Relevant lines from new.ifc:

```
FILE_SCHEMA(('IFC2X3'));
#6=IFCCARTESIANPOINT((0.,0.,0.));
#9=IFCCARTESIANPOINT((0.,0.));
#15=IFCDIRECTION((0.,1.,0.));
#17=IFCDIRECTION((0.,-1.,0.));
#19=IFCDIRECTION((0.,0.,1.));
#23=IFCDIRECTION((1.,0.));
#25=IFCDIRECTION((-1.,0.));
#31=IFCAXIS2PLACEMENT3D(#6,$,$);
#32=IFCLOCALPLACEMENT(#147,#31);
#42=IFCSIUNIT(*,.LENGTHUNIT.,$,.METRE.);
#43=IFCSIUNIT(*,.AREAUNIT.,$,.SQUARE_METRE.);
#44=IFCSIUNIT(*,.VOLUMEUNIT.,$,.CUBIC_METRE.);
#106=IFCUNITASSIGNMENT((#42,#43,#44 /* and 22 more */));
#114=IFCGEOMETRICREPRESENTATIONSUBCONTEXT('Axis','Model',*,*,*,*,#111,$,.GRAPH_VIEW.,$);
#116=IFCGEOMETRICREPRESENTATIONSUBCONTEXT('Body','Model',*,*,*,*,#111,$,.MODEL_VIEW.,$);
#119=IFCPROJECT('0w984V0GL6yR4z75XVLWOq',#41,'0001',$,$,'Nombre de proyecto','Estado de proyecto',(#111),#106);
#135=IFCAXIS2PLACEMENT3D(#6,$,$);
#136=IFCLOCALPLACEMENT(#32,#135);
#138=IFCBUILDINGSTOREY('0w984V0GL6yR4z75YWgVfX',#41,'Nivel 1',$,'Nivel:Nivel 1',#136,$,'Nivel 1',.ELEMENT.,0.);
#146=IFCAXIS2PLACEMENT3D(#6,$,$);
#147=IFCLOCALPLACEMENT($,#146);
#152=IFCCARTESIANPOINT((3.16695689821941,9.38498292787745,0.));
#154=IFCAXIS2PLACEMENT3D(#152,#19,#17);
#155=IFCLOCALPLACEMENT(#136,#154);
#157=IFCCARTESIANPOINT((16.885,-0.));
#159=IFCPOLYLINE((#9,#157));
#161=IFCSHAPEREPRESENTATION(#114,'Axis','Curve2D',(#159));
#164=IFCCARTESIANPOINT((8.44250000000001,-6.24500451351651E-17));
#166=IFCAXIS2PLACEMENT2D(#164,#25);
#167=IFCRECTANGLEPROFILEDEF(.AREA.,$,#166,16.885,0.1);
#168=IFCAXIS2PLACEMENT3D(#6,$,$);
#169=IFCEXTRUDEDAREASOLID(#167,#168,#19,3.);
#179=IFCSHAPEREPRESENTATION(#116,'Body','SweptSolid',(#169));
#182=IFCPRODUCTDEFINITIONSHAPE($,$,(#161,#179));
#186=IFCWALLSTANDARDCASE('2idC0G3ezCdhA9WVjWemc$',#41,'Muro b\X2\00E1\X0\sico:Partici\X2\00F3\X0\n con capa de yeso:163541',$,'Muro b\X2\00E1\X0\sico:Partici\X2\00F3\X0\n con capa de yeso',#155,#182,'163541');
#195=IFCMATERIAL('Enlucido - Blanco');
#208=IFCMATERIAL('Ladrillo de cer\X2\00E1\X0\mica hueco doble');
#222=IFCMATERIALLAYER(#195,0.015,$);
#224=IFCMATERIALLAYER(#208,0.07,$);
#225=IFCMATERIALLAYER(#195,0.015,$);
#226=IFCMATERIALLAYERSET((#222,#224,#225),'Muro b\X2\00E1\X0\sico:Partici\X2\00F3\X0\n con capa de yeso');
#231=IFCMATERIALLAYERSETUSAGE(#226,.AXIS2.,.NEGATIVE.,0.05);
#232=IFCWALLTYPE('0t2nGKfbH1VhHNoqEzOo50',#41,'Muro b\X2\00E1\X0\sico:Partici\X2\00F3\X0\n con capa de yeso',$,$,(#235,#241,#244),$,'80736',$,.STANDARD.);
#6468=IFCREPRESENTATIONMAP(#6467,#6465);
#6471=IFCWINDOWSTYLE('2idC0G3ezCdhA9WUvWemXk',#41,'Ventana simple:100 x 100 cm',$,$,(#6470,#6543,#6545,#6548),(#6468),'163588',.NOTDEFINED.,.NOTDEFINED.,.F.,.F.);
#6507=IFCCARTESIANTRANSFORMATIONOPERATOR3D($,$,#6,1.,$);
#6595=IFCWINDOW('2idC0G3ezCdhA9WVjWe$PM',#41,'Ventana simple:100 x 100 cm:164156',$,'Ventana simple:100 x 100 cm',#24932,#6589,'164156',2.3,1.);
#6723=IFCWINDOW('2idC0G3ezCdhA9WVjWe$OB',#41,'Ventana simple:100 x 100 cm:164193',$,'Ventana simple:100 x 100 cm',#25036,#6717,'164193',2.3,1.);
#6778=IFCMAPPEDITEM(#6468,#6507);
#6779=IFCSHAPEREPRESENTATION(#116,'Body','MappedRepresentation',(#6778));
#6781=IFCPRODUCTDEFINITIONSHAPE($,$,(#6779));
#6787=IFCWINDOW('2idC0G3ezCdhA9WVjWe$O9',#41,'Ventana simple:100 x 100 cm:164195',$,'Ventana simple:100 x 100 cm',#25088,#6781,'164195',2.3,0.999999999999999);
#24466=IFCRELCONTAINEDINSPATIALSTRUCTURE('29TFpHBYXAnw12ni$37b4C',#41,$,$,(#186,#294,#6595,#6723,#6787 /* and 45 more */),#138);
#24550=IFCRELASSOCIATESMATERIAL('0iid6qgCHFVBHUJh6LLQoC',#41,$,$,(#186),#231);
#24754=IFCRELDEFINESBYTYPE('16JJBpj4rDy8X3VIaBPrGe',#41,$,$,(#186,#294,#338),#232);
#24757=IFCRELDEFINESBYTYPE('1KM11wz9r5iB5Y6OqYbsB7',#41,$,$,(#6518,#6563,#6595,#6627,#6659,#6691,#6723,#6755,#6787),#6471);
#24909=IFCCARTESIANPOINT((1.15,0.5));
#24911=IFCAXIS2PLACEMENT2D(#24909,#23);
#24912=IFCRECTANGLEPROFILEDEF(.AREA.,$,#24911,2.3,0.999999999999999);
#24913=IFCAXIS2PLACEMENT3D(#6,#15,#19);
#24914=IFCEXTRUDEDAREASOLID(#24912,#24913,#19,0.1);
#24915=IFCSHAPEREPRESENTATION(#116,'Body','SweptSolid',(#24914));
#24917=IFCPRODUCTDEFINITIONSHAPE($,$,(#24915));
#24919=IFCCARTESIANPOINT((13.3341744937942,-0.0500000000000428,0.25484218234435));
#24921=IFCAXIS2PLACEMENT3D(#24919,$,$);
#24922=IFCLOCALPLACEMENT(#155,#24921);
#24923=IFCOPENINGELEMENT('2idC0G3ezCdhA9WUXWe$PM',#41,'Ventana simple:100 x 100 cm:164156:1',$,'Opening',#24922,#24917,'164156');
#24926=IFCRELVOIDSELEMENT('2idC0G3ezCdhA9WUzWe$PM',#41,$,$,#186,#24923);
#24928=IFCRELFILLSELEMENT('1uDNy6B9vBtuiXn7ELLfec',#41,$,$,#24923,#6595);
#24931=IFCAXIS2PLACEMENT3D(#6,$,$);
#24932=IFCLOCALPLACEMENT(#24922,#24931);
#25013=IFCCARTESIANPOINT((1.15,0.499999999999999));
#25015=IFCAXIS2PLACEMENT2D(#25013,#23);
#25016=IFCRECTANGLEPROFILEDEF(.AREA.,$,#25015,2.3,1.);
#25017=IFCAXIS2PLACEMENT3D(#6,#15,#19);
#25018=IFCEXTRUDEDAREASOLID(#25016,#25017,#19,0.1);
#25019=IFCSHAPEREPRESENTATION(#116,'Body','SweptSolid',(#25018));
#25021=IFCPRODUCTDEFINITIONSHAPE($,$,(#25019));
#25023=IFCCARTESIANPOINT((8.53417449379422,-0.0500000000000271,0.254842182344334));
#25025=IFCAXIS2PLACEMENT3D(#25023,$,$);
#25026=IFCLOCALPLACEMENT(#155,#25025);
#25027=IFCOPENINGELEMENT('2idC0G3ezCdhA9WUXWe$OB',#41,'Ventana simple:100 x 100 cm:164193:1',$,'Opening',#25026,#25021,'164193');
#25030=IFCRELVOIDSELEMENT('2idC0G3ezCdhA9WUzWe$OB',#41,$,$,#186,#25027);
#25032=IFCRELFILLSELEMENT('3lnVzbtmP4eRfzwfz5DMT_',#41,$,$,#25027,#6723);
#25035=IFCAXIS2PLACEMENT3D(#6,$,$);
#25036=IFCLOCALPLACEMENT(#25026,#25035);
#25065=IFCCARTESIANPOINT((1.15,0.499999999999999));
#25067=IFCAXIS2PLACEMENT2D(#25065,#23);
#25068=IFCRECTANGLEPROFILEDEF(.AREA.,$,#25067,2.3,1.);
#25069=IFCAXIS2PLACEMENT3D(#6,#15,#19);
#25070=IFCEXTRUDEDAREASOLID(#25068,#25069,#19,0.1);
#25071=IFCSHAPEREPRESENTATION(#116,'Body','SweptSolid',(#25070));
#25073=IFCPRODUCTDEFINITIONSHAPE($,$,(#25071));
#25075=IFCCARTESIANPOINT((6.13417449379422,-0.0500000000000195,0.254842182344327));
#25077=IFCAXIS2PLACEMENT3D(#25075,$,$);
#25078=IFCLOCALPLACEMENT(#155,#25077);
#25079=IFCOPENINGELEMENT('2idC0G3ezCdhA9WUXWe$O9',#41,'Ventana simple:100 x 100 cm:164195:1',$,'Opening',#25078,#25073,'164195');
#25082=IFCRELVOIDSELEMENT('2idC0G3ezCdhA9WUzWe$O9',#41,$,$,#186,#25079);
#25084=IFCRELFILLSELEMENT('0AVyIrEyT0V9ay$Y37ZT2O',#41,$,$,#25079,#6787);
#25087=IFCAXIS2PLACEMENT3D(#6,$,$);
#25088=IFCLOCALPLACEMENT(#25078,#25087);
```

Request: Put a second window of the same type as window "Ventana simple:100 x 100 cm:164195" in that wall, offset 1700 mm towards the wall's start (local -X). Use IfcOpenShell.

```python
import ifcopenshell
import ifcopenshell.api.feature
import ifcopenshell.api.geometry
import ifcopenshell.api.root
import ifcopenshell.geom
import ifcopenshell.util.element
import ifcopenshell.util.placement
import ifcopenshell.util.shape

model = ifcopenshell.open("new.ifc")
settings = ifcopenshell.geom.settings()


def volume(element):
    """Net volume in cubic metres, openings subtracted."""
    shape = ifcopenshell.geom.create_shape(settings, element)
    return ifcopenshell.util.shape.get_volume(shape.geometry)


def reuse_history(source, copy):
    """copy_class also copies each property set's owner history, people and application; keep the originals."""
    for rel in copy.IsDefinedBy:
        if rel.is_a("IfcRelDefinesByProperties") and (history := rel.RelatingPropertyDefinition.OwnerHistory):
            rel.RelatingPropertyDefinition.OwnerHistory = source.OwnerHistory
            ifcopenshell.util.element.remove_deep2(model, history)


window = model.by_id(6787)
opening = window.FillsVoids[0].RelatingOpeningElement
wall = opening.VoidsElements[0].RelatingBuildingElement
before = volume(wall)
shift = ifcopenshell.util.placement.get_local_placement(wall.ObjectPlacement)[:3, 0] * -1.7

# copy_class copies the void relationship, type, container and properties, but no geometry.
new_opening = ifcopenshell.api.root.copy_class(model, product=opening)
new_opening.Representation = ifcopenshell.util.element.copy_deep(
    model, opening.Representation, exclude=["IfcGeometricRepresentationContext", "IfcRepresentationMap"]
)
new_opening.Name = "Ventana simple:100 x 100 cm"
new_opening.Tag = None
new_window = ifcopenshell.api.root.copy_class(model, product=window)
new_window.Representation = ifcopenshell.util.element.copy_deep(
    model, window.Representation, exclude=["IfcGeometricRepresentationContext", "IfcRepresentationMap"]
)
new_window.Name = "Ventana simple:100 x 100 cm"
new_window.Tag = None
reuse_history(window, new_window)
fills = ifcopenshell.api.feature.add_filling(model, opening=new_opening, element=new_window)
fills.OwnerHistory = new_window.OwnerHistory  # required in IFC2X3

for old, new in ((opening, new_opening), (window, new_window)):
    matrix = ifcopenshell.util.placement.get_local_placement(old.ObjectPlacement)
    matrix[:3, 3] += shift
    ifcopenshell.api.geometry.edit_object_placement(model, product=new, matrix=matrix, is_si=False)

after = volume(wall)

print(f"wall volume {before:.3f} -> {after:.3f} m3")

model.write("new_v2.ifc")
```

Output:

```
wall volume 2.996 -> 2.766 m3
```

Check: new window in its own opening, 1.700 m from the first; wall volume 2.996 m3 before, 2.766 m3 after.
